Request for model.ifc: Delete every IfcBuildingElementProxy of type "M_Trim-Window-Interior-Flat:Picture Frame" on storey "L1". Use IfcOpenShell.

First a look at what the model holds.

```python
import ifcopenshell
import ifcopenshell.util.element

model = ifcopenshell.open("model.ifc")
print(model.schema)
storey = next(s for s in model.by_type("IfcBuildingStorey") if s.Name == "L1")
proxies = [e for e in ifcopenshell.util.element.get_decomposition(storey) if e.is_a("IfcBuildingElementProxy")]
seen = {}
for e in proxies:
    element_type = ifcopenshell.util.element.get_type(e)
    name = element_type.Name if element_type not in (None, e) else None
    seen[name] = seen.get(name, 0) + 1
for name, count in sorted(seen.items(), key=str):
    print(count, "x", name)
```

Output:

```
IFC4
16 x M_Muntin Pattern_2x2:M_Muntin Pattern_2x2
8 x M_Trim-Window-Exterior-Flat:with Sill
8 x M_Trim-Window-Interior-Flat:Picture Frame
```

```python
import ifcopenshell
import ifcopenshell.api.root
import ifcopenshell.util.element

model = ifcopenshell.open("model.ifc")

storey = next(s for s in model.by_type("IfcBuildingStorey") if s.Name == "L1")
proxies = [e for e in ifcopenshell.util.element.get_decomposition(storey) if e.is_a("IfcBuildingElementProxy")]
targets = [e for e in proxies if (t := ifcopenshell.util.element.get_type(e)) not in (None, e) and t.Name == "M_Trim-Window-Interior-Flat:Picture Frame"]

for e in targets:
    ifcopenshell.api.root.remove_product(model, product=e)
print(len(targets), "removed")

model.write("model_edited.ifc")
```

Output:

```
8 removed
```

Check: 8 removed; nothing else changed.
